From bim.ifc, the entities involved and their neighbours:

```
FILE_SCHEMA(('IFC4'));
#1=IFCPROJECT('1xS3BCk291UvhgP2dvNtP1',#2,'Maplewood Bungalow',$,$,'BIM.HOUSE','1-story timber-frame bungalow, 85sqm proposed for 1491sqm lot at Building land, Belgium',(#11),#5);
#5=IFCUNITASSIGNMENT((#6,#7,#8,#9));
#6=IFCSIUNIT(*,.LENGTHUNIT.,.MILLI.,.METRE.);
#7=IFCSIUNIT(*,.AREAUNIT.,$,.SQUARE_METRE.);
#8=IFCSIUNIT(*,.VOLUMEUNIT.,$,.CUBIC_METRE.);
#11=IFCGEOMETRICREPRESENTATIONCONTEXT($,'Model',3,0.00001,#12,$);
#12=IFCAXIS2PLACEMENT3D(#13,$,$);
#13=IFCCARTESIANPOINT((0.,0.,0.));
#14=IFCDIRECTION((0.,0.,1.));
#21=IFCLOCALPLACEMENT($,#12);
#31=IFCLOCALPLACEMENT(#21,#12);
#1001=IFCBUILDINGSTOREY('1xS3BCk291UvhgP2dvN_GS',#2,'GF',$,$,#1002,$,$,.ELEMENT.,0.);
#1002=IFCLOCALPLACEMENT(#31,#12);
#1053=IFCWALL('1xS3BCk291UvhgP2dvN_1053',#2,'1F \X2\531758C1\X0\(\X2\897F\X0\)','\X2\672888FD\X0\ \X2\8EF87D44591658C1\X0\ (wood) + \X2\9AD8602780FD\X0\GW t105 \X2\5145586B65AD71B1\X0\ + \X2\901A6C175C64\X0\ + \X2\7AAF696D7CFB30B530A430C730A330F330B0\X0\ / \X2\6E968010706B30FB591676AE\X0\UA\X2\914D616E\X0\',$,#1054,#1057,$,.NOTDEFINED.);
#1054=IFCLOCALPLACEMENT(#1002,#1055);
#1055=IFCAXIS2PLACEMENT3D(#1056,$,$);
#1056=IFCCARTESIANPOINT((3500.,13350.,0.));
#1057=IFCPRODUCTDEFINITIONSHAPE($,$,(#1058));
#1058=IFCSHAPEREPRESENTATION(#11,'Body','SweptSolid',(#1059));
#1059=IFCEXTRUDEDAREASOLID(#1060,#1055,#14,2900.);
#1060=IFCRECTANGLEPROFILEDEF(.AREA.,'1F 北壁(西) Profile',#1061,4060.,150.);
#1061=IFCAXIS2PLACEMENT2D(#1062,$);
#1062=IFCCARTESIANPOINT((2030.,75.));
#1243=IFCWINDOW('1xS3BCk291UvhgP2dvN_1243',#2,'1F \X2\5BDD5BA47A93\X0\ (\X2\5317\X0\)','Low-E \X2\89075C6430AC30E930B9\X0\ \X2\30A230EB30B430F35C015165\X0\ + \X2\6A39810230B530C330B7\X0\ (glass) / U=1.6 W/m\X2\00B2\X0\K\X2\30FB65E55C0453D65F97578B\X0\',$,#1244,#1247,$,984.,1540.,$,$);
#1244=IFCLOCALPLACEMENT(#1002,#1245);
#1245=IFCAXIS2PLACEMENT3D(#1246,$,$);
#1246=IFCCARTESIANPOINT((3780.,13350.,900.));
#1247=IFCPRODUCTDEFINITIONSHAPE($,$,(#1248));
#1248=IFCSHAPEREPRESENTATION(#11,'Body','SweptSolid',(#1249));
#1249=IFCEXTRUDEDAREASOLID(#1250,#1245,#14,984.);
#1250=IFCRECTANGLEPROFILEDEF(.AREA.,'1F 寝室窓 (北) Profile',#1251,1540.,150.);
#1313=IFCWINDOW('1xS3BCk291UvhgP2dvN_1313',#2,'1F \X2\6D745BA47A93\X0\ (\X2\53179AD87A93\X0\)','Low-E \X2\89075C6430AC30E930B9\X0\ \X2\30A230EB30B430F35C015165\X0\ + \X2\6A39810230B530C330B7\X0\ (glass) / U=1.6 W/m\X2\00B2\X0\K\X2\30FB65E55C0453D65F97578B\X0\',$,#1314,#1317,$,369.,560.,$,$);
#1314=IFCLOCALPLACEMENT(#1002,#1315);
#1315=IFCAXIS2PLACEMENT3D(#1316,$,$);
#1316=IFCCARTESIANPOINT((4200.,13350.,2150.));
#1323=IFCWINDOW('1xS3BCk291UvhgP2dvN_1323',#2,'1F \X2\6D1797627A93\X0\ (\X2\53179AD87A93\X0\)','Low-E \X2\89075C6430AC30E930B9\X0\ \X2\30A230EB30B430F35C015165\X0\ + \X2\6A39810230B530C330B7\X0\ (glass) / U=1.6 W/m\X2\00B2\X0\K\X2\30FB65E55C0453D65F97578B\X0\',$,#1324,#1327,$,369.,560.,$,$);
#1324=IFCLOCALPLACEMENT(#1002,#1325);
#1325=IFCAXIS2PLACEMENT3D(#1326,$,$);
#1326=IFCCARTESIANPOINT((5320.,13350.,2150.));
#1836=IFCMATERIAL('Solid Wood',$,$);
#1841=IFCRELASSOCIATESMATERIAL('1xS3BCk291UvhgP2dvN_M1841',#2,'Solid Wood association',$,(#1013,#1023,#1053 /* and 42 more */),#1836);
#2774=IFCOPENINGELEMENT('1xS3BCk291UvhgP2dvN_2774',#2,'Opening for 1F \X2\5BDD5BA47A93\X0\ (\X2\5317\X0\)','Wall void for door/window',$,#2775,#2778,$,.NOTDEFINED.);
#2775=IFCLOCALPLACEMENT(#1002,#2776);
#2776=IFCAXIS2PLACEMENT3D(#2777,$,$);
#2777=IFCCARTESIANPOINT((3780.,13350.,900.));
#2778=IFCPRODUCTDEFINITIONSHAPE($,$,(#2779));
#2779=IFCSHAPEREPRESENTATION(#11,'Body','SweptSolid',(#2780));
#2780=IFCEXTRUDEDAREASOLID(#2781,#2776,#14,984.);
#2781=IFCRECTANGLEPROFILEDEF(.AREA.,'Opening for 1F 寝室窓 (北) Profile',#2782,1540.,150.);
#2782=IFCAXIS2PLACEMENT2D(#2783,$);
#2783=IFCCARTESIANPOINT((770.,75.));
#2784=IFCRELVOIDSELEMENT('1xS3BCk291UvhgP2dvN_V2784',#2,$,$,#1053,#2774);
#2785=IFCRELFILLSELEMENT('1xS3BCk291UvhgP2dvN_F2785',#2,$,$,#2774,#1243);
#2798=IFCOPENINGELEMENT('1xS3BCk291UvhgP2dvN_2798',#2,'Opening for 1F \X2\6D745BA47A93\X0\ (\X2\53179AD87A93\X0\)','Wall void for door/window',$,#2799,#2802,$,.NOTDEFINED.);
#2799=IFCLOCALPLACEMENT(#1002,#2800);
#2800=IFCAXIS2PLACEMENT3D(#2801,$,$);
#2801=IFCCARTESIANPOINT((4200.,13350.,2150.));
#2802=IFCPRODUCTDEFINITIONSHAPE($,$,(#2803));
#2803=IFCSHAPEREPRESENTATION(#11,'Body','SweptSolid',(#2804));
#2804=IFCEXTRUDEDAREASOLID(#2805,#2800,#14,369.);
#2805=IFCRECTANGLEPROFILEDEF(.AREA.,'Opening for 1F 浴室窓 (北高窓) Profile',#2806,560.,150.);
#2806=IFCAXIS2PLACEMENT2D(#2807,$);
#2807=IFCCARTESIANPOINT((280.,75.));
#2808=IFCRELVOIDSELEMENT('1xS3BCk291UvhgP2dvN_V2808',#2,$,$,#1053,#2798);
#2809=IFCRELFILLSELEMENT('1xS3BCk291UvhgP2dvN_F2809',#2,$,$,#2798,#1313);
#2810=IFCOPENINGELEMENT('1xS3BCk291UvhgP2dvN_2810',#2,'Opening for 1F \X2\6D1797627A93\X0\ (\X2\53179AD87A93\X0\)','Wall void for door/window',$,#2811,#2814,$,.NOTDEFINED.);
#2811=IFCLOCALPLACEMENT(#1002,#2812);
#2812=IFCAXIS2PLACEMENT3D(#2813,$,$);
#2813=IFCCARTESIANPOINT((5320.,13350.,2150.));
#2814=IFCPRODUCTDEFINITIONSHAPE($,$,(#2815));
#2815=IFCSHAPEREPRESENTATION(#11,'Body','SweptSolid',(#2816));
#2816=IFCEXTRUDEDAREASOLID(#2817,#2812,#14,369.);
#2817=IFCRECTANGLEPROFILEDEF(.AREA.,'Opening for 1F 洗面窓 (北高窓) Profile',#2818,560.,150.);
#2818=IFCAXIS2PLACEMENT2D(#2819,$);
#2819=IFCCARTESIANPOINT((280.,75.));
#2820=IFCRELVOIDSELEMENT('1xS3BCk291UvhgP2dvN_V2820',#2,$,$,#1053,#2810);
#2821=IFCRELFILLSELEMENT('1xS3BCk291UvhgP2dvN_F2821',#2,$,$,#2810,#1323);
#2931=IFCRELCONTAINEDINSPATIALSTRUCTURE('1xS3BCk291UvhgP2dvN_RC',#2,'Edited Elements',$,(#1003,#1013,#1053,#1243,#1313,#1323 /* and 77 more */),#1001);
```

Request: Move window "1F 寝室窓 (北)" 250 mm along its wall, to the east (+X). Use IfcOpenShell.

```python
import ifcopenshell
import ifcopenshell.api.geometry
import ifcopenshell.util.placement
import ifcopenshell.util.unit

model = ifcopenshell.open("bim.ifc")
unit_scale = ifcopenshell.util.unit.calculate_unit_scale(model)

window = model.by_guid("1xS3BCk291UvhgP2dvN_1243")
opening = window.FillsVoids[0].RelatingOpeningElement
wall = opening.VoidsElements[0].RelatingBuildingElement

wall_matrix = ifcopenshell.util.placement.get_local_placement(wall.ObjectPlacement)
shift = wall_matrix[:3, 0] * 0.25 / unit_scale
before = ifcopenshell.util.placement.get_local_placement(window.ObjectPlacement)[:3, 3].copy()

# The window is not placed relative to its opening, so move both.
for product in (opening, window):
    matrix = ifcopenshell.util.placement.get_local_placement(product.ObjectPlacement)
    matrix[:3, 3] += shift
    ifcopenshell.api.geometry.edit_object_placement(model, product=product, matrix=matrix, is_si=False)

after = ifcopenshell.util.placement.get_local_placement(window.ObjectPlacement)[:3, 3]
print("window moved by", (after - before).round(3) + 0.0)

model.write("bim_edited.ifc")
```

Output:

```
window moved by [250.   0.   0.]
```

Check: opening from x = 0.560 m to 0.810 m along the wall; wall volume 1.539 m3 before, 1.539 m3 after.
